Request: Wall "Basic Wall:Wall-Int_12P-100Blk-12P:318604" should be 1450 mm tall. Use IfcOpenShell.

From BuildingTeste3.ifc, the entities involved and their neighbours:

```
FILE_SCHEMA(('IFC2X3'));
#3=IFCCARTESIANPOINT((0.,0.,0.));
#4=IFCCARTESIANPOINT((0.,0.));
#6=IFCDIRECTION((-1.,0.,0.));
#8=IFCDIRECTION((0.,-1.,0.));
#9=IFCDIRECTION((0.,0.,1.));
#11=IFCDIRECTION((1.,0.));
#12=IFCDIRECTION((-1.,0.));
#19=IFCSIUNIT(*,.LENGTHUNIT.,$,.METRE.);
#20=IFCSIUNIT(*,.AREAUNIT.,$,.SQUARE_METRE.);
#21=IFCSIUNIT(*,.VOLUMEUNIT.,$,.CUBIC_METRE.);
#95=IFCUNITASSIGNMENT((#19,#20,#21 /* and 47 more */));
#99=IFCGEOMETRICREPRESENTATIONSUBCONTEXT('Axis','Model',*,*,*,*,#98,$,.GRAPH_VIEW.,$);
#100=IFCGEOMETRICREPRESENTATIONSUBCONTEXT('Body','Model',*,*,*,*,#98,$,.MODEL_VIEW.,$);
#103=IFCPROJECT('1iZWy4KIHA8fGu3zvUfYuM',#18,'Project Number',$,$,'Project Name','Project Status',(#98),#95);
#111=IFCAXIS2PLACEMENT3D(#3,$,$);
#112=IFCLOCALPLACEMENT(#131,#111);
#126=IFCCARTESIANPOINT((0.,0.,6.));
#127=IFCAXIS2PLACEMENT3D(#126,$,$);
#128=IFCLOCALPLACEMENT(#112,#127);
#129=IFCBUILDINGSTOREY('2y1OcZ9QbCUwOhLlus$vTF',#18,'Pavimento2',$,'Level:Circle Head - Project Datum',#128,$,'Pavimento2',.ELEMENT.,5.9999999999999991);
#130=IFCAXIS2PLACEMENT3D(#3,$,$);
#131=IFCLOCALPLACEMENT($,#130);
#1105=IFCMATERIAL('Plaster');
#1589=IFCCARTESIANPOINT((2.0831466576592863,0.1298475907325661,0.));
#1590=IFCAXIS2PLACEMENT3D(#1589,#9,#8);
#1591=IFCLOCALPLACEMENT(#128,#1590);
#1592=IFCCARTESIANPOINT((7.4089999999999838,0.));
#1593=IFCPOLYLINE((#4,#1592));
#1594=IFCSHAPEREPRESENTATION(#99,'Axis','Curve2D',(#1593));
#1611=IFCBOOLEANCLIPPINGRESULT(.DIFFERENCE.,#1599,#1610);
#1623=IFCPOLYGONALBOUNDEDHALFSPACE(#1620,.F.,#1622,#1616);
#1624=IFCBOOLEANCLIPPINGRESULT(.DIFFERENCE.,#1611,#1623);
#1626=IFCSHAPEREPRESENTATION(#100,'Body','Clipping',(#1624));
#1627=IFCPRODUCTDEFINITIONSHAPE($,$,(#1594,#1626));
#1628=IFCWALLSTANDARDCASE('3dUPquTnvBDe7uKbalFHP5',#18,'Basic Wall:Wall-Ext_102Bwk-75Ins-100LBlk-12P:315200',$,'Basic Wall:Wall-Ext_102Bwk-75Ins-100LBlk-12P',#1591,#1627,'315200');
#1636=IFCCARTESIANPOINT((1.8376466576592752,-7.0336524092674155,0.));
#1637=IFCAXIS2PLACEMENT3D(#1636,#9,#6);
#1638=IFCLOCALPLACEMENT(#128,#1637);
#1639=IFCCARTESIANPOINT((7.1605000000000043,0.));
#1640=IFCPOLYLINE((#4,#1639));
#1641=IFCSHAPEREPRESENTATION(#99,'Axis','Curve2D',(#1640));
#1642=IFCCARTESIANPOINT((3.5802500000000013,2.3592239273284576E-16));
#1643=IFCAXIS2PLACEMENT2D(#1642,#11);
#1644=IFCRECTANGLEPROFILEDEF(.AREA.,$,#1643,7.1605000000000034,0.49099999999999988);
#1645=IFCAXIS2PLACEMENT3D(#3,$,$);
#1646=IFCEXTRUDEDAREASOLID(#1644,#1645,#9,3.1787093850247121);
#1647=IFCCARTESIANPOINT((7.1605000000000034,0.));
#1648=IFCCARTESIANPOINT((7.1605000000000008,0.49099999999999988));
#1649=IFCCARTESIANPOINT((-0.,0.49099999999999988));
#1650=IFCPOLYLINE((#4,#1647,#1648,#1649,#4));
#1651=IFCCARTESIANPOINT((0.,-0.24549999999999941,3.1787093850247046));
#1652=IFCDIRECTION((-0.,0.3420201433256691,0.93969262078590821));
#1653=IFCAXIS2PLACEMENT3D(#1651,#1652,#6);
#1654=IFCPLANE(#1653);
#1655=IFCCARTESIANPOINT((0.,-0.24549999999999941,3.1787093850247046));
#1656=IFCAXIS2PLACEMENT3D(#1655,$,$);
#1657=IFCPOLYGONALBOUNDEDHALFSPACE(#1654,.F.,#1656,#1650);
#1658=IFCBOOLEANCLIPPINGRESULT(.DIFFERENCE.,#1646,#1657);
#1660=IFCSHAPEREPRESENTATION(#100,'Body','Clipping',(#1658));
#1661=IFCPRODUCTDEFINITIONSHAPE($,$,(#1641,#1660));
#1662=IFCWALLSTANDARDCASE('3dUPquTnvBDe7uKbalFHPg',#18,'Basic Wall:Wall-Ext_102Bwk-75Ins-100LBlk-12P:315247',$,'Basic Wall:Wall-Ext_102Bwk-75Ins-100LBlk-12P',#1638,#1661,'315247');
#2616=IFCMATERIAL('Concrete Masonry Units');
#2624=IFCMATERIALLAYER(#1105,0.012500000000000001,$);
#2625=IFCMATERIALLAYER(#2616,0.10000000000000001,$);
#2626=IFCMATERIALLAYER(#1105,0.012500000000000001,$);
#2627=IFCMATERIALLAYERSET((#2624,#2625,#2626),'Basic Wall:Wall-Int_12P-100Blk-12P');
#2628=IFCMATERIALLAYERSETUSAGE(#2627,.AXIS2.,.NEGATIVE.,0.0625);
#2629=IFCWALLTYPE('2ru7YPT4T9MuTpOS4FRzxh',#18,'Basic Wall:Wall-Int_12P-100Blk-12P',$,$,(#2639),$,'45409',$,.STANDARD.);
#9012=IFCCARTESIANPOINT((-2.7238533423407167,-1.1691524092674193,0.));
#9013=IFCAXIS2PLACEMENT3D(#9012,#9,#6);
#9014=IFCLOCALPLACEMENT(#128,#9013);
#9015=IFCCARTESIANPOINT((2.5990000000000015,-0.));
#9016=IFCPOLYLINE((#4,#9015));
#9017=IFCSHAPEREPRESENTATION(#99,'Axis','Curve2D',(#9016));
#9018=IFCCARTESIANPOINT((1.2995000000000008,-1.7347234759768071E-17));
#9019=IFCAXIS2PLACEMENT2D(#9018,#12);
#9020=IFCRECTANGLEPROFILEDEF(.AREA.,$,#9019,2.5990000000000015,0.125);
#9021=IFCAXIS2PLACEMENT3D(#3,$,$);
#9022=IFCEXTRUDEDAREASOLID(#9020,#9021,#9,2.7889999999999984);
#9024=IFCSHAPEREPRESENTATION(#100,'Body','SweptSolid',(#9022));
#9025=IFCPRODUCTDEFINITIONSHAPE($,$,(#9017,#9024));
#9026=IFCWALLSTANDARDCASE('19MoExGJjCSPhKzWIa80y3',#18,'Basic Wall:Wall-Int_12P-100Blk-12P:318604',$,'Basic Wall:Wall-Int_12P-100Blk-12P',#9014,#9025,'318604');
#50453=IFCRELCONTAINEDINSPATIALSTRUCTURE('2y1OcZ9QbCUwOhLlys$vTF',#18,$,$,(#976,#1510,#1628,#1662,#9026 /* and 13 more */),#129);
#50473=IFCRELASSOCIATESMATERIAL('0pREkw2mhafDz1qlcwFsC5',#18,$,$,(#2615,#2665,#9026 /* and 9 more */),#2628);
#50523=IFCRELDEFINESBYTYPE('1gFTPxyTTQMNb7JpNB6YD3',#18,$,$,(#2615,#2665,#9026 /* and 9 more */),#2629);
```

```python
import ifcopenshell
import ifcopenshell.geom
import ifcopenshell.util.representation
import ifcopenshell.util.shape

model = ifcopenshell.open("BuildingTeste3.ifc")
settings = ifcopenshell.geom.settings()


def volume(element):
    """Net volume in cubic metres, openings subtracted."""
    shape = ifcopenshell.geom.create_shape(settings, element)
    return ifcopenshell.util.shape.get_volume(shape.geometry)


wall = model.by_id(9026)
before = volume(wall)

body = ifcopenshell.util.representation.get_representation(wall, "Model", "Body")
solid = body.Items[0]
old_height = solid.Depth
solid.Depth = 1.45
after = volume(wall)

print(f"height {old_height:g} -> {solid.Depth:g}, volume {before:.3f} -> {after:.3f} m3")

model.write("BuildingTeste3_edited.ifc")
```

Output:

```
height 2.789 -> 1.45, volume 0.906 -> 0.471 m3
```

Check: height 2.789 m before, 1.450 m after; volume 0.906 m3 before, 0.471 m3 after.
